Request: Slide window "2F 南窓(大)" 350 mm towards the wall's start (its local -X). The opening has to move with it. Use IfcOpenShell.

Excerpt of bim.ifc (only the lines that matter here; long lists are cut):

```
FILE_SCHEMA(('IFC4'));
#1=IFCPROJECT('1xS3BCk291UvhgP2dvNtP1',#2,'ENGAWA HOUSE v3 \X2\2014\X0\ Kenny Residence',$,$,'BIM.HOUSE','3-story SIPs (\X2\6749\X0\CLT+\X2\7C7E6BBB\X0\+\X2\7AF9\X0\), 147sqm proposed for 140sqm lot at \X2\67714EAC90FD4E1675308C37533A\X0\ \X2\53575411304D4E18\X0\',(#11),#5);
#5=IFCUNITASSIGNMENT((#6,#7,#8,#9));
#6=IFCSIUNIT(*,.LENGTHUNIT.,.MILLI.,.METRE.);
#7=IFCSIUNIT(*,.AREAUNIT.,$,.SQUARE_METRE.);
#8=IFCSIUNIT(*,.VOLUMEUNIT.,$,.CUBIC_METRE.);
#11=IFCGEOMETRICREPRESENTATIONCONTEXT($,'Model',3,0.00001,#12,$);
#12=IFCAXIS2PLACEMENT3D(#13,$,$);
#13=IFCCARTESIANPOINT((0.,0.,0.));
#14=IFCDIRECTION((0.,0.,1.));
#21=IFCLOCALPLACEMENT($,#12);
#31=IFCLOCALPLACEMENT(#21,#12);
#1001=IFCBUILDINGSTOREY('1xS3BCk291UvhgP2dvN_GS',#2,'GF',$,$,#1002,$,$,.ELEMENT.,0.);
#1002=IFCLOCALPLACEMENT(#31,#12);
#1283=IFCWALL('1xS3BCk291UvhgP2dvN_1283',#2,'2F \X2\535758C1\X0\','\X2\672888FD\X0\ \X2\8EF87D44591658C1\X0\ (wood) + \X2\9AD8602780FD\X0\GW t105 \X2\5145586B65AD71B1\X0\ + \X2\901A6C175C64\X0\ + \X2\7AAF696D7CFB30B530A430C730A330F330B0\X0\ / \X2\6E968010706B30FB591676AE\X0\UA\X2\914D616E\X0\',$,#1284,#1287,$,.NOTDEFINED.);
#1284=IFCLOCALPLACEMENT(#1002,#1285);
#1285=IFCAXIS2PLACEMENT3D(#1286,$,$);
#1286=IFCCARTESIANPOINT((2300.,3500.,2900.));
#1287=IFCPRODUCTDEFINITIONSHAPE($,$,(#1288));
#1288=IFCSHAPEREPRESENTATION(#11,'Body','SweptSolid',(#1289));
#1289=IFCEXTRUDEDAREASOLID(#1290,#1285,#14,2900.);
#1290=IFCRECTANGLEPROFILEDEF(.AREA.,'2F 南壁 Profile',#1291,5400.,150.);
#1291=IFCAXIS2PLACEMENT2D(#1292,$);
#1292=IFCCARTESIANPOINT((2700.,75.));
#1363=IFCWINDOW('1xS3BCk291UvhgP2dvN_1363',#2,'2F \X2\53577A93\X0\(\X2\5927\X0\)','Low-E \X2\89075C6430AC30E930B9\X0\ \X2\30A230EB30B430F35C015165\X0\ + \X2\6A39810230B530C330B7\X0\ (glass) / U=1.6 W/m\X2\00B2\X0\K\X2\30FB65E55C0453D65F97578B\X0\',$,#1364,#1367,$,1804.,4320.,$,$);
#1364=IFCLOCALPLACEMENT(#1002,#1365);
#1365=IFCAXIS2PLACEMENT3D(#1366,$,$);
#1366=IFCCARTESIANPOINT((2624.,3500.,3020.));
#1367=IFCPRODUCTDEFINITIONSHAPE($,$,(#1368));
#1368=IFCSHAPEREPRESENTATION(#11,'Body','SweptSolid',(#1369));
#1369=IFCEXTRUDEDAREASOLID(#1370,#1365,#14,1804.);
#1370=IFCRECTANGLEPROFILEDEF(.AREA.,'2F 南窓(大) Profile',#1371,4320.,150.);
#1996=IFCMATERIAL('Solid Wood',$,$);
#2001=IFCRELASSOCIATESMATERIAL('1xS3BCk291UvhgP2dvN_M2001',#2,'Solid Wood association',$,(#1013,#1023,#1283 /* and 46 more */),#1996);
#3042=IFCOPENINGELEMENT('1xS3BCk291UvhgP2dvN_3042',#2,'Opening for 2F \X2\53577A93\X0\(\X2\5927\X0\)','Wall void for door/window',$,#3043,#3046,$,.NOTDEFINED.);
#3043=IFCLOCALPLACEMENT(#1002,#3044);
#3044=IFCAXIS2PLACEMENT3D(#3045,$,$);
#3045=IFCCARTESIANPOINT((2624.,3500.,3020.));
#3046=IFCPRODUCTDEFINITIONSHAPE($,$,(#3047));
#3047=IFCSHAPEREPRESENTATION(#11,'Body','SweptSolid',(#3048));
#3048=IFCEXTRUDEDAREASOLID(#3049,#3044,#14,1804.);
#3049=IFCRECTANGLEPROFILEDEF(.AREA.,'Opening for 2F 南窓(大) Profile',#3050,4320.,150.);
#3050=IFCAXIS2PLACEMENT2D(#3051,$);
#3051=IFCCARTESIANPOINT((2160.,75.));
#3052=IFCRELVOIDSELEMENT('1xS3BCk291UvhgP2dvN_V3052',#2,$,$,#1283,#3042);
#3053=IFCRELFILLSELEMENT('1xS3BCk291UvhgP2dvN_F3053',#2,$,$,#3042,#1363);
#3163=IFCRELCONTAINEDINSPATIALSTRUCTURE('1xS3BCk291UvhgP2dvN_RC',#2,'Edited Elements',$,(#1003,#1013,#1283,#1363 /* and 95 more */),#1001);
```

```python
import ifcopenshell
import ifcopenshell.api.geometry
import ifcopenshell.util.placement

model = ifcopenshell.open("bim.ifc")

window = model.by_id(1363)
opening = window.FillsVoids[0].RelatingOpeningElement
wall = opening.VoidsElements[0].RelatingBuildingElement

wall_matrix = ifcopenshell.util.placement.get_local_placement(wall.ObjectPlacement)
shift = wall_matrix[:3, 0] * -350.0
before = ifcopenshell.util.placement.get_local_placement(window.ObjectPlacement)[:3, 3].copy()

# The window is not placed relative to its opening, so move both.
for product in (opening, window):
    matrix = ifcopenshell.util.placement.get_local_placement(product.ObjectPlacement)
    matrix[:3, 3] += shift
    ifcopenshell.api.geometry.edit_object_placement(model, product=product, matrix=matrix, is_si=False)

after = ifcopenshell.util.placement.get_local_placement(window.ObjectPlacement)[:3, 3]
print("window moved by", (after - before).round(3) + 0.0)

model.write("bim_v2.ifc")
```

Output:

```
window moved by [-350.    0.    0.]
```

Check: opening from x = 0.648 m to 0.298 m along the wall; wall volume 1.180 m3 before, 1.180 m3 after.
